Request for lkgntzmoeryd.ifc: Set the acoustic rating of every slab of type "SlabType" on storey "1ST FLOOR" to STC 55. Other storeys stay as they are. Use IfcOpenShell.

First a look at what the model holds.

```python
import ifcopenshell
import ifcopenshell.util.element

model = ifcopenshell.open("lkgntzmoeryd.ifc")
print(model.schema)
storey = next(s for s in model.by_type("IfcBuildingStorey") if s.Name == "1ST FLOOR")
slabs = [e for e in ifcopenshell.util.element.get_decomposition(storey) if e.is_a("IfcSlab")]
seen = {}
for e in slabs:
    element_type = ifcopenshell.util.element.get_type(e)
    key = (element_type.Name if element_type != e and element_type else None, ifcopenshell.util.element.get_pset(e, "Pset_SlabCommon", "AcousticRating"))
    seen[key] = seen.get(key, 0) + 1
for (name, value), count in sorted(seen.items(), key=str):
    print(count, "x", name, "|", value)
```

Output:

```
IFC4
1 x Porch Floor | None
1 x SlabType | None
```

```python
import ifcopenshell
import ifcopenshell.api.pset
import ifcopenshell.util.element

model = ifcopenshell.open("lkgntzmoeryd.ifc")

storey = next(s for s in model.by_type("IfcBuildingStorey") if s.Name == "1ST FLOOR")
slabs = [e for e in ifcopenshell.util.element.get_decomposition(storey) if e.is_a("IfcSlab")]

count = 0
for e in slabs:
    element_type = ifcopenshell.util.element.get_type(e)
    if element_type in (None, e) or element_type.Name != "SlabType":
        continue
    # add_pset returns the element's existing set when there is one.
    pset = ifcopenshell.api.pset.add_pset(model, product=e, name="Pset_SlabCommon")
    ifcopenshell.api.pset.edit_pset(model, pset=pset, properties={"AcousticRating": "STC 55"})
    count += 1

print(count, "slabs updated")

model.write("lkgntzmoeryd-out.ifc")
```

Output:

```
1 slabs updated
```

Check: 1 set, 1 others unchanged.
